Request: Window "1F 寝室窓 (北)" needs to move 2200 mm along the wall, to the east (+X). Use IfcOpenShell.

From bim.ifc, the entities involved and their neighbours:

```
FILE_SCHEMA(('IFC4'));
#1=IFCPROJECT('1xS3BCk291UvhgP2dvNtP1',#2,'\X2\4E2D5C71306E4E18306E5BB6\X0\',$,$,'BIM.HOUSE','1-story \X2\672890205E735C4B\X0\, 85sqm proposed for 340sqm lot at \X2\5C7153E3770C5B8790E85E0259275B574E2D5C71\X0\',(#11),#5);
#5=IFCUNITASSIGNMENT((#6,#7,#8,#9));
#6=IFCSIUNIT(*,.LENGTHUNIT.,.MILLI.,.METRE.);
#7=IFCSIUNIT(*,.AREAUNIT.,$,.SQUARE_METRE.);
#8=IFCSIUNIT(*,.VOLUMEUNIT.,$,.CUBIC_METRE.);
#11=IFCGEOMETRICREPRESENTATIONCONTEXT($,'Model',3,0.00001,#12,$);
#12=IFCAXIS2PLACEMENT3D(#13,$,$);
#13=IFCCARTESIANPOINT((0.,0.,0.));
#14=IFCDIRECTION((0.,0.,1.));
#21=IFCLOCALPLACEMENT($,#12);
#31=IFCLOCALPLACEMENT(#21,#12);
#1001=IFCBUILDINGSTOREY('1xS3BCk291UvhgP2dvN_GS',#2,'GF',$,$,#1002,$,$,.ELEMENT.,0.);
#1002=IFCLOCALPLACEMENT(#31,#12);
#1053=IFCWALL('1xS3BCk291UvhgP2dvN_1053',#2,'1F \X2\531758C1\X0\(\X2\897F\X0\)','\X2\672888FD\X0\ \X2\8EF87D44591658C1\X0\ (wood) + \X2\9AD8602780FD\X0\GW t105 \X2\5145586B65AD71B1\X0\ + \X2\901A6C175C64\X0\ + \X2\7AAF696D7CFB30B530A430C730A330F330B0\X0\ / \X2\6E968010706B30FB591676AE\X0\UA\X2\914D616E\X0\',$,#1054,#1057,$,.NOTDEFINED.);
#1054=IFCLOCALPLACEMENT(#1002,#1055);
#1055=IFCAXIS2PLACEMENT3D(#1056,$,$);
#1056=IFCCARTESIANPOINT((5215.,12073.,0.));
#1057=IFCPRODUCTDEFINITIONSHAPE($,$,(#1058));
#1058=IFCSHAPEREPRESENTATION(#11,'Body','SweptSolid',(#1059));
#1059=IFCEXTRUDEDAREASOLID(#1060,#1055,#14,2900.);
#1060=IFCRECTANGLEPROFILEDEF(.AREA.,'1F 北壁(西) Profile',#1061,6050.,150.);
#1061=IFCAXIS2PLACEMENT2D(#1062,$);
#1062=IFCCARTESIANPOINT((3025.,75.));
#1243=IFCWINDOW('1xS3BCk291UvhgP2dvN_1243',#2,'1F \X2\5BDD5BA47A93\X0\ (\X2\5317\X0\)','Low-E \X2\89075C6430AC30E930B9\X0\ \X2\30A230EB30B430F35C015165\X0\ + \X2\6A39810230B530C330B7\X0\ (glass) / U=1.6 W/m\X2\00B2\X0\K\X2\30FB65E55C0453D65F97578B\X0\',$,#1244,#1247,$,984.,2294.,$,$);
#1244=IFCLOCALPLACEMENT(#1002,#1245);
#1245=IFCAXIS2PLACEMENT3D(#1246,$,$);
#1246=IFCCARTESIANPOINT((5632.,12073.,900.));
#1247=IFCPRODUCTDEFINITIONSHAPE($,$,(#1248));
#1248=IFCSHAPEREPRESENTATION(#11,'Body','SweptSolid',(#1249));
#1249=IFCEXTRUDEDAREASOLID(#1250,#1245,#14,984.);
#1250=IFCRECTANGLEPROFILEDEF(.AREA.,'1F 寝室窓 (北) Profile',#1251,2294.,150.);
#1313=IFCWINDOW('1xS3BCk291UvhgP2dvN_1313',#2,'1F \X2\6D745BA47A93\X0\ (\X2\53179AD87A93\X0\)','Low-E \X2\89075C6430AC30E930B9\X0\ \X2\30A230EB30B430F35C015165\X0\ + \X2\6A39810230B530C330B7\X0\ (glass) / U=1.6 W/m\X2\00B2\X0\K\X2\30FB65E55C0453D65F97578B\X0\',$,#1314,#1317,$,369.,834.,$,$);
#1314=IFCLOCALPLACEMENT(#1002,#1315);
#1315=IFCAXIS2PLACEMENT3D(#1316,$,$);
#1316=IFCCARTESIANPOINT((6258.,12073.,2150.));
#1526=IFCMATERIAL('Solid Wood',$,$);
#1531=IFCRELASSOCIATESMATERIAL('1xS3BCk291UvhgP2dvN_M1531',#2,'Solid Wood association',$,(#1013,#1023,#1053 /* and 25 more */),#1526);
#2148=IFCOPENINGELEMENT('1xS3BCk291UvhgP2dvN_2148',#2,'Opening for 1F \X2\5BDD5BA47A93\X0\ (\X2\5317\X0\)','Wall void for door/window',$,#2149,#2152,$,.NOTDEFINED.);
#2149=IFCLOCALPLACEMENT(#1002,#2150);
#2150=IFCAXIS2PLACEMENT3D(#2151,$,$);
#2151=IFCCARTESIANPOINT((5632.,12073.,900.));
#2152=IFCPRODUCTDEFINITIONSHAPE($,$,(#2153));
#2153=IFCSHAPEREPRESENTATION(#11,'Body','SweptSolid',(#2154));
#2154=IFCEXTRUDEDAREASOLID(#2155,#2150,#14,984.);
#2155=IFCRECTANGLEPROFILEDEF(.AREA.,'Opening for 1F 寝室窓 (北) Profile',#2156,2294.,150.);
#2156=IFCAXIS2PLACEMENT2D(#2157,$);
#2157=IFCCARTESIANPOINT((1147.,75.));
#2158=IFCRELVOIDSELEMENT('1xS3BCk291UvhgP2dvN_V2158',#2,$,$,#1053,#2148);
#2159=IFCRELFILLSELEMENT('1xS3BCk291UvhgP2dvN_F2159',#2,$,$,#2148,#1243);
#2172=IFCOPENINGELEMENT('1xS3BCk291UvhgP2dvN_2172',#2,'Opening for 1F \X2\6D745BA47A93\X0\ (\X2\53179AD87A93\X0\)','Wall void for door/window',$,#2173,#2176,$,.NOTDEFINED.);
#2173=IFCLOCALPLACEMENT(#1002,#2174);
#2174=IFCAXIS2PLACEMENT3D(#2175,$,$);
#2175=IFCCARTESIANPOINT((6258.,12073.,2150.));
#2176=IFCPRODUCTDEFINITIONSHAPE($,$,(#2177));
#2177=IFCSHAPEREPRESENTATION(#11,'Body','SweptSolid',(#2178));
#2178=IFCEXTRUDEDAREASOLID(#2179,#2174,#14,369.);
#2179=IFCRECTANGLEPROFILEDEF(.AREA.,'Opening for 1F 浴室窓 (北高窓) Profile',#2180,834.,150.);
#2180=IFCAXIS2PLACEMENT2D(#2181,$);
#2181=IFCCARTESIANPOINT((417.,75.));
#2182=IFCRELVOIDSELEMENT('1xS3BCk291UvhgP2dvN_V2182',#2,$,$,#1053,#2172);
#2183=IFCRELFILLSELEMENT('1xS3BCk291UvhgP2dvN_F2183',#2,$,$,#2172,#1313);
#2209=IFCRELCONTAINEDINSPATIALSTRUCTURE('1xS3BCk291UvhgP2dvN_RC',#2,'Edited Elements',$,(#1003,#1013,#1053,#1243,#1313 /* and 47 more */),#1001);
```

```python
import ifcopenshell
import ifcopenshell.api.geometry
import ifcopenshell.util.placement

model = ifcopenshell.open("bim.ifc")

window = model.by_guid("1xS3BCk291UvhgP2dvN_1243")
opening = window.FillsVoids[0].RelatingOpeningElement
wall = opening.VoidsElements[0].RelatingBuildingElement

wall_matrix = ifcopenshell.util.placement.get_local_placement(wall.ObjectPlacement)
shift = wall_matrix[:3, 0] * 2200.0
before = ifcopenshell.util.placement.get_local_placement(window.ObjectPlacement)[:3, 3].copy()

# The window is not placed relative to its opening, so move both.
for product in (opening, window):
    matrix = ifcopenshell.util.placement.get_local_placement(product.ObjectPlacement)
    matrix[:3, 3] += shift
    ifcopenshell.api.geometry.edit_object_placement(model, product=product, matrix=matrix, is_si=False)

after = ifcopenshell.util.placement.get_local_placement(window.ObjectPlacement)[:3, 3]
print("window moved by", (after - before).round(3) + 0.0)

model.write("bim_rev.ifc")
```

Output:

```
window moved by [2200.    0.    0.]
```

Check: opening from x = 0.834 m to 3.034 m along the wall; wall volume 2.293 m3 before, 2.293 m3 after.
